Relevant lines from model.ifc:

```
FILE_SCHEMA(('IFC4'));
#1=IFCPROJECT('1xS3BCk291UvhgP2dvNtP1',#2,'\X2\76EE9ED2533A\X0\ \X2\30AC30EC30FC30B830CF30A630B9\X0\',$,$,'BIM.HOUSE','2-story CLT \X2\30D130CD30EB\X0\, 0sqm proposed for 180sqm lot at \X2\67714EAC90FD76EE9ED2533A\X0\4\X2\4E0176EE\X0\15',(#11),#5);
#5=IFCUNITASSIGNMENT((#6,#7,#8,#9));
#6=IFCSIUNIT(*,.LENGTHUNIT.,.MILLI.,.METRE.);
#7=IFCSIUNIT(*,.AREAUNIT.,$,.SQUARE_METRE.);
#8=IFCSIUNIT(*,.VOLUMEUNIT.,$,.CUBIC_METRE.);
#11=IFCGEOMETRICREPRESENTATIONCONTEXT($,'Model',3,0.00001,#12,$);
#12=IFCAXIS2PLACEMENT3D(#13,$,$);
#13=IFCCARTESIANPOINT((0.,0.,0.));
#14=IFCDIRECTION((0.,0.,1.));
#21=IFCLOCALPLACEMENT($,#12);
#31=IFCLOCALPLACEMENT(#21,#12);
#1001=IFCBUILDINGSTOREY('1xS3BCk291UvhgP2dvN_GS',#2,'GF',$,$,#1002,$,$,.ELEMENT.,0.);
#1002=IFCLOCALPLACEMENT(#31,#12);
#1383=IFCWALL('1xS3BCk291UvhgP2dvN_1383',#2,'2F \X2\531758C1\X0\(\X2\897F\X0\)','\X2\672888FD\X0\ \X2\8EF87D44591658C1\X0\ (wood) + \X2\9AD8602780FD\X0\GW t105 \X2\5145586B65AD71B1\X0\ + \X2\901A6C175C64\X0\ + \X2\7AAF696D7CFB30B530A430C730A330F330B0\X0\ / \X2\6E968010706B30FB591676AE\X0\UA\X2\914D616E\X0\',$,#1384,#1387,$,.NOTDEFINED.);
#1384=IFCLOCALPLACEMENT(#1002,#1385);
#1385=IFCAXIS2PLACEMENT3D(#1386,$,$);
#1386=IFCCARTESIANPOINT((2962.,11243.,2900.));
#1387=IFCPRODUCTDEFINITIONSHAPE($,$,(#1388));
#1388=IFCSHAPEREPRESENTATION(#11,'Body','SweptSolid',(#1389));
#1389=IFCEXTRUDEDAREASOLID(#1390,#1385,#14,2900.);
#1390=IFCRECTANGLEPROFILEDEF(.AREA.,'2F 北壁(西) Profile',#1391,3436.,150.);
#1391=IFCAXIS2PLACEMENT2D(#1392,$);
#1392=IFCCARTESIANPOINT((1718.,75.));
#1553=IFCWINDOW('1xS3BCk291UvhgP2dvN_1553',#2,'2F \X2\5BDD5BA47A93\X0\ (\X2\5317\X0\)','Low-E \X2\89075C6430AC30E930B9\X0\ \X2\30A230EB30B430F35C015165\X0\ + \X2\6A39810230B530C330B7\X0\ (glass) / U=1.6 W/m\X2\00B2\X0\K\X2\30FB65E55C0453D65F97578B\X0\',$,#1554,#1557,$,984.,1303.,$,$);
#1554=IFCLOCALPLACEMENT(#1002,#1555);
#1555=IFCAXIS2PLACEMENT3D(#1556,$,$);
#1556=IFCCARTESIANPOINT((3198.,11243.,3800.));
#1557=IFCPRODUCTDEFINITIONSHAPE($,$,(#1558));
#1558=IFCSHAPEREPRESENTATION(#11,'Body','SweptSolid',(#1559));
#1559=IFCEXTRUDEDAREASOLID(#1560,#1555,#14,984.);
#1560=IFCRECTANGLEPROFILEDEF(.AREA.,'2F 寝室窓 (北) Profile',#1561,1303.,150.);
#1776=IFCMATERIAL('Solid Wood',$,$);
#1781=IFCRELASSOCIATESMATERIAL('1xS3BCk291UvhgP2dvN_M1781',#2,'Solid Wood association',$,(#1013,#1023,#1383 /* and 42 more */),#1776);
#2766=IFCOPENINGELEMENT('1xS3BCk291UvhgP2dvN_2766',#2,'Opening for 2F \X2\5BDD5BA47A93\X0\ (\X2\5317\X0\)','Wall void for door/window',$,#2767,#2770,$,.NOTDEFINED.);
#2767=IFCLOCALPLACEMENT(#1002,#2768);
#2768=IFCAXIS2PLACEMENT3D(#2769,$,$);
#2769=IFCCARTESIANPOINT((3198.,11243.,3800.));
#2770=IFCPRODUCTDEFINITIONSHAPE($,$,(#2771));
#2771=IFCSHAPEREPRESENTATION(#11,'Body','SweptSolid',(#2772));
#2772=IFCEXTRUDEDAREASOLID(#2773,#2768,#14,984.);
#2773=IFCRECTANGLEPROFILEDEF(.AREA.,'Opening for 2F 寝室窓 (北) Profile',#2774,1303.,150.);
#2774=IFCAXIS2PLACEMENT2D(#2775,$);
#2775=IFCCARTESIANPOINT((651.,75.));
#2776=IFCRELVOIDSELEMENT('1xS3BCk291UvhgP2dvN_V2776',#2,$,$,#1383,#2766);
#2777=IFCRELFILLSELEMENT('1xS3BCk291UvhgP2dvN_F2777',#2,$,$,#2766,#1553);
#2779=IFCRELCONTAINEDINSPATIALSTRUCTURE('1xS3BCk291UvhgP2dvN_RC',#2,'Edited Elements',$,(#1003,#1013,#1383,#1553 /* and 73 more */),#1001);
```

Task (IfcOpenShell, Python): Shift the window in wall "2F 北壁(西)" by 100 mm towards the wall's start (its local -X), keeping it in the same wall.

```python
import ifcopenshell
import ifcopenshell.api.geometry
import ifcopenshell.util.placement

model = ifcopenshell.open("model.ifc")

window = model.by_guid("1xS3BCk291UvhgP2dvN_1553")
opening = window.FillsVoids[0].RelatingOpeningElement
wall = opening.VoidsElements[0].RelatingBuildingElement

wall_matrix = ifcopenshell.util.placement.get_local_placement(wall.ObjectPlacement)
shift = wall_matrix[:3, 0] * -100.0
before = ifcopenshell.util.placement.get_local_placement(window.ObjectPlacement)[:3, 3].copy()

# The window is not placed relative to its opening, so move both.
for product in (opening, window):
    matrix = ifcopenshell.util.placement.get_local_placement(product.ObjectPlacement)
    matrix[:3, 3] += shift
    ifcopenshell.api.geometry.edit_object_placement(model, product=product, matrix=matrix, is_si=False)

after = ifcopenshell.util.placement.get_local_placement(window.ObjectPlacement)[:3, 3]
print("window moved by", (after - before).round(3) + 0.0)

model.write("model_rev.ifc")
```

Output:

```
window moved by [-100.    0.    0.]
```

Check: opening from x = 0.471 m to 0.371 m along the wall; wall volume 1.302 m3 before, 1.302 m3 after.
